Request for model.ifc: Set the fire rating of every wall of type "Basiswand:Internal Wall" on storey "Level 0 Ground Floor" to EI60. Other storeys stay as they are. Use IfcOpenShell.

First a look at what the model holds.

```python
import ifcopenshell
import ifcopenshell.util.element

model = ifcopenshell.open("model.ifc")
print(model.schema)
storey = next(s for s in model.by_type("IfcBuildingStorey") if s.Name == "Level 0 Ground Floor")
walls = [e for e in ifcopenshell.util.element.get_decomposition(storey) if e.is_a("IfcWall")]
seen = {}
for e in walls:
    element_type = ifcopenshell.util.element.get_type(e)
    key = (element_type.Name if element_type != e and element_type else None, ifcopenshell.util.element.get_pset(e, "Pset_WallCommon", "FireRating"))
    seen[key] = seen.get(key, 0) + 1
for (name, value), count in sorted(seen.items(), key=str):
    print(count, "x", name, "|", value)
```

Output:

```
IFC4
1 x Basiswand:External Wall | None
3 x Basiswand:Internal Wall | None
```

```python
import ifcopenshell
import ifcopenshell.api.pset
import ifcopenshell.util.element

model = ifcopenshell.open("model.ifc")

storey = next(s for s in model.by_type("IfcBuildingStorey") if s.Name == "Level 0 Ground Floor")
walls = [e for e in ifcopenshell.util.element.get_decomposition(storey) if e.is_a("IfcWall")]

count = 0
for e in walls:
    element_type = ifcopenshell.util.element.get_type(e)
    if element_type in (None, e) or element_type.Name != "Basiswand:Internal Wall":
        continue
    # add_pset returns the element's existing set when there is one.
    pset = ifcopenshell.api.pset.add_pset(model, product=e, name="Pset_WallCommon")
    ifcopenshell.api.pset.edit_pset(model, pset=pset, properties={"FireRating": "EI60"})
    count += 1

print(count, "walls updated")

model.write("model_updated.ifc")
```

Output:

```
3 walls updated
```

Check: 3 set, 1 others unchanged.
